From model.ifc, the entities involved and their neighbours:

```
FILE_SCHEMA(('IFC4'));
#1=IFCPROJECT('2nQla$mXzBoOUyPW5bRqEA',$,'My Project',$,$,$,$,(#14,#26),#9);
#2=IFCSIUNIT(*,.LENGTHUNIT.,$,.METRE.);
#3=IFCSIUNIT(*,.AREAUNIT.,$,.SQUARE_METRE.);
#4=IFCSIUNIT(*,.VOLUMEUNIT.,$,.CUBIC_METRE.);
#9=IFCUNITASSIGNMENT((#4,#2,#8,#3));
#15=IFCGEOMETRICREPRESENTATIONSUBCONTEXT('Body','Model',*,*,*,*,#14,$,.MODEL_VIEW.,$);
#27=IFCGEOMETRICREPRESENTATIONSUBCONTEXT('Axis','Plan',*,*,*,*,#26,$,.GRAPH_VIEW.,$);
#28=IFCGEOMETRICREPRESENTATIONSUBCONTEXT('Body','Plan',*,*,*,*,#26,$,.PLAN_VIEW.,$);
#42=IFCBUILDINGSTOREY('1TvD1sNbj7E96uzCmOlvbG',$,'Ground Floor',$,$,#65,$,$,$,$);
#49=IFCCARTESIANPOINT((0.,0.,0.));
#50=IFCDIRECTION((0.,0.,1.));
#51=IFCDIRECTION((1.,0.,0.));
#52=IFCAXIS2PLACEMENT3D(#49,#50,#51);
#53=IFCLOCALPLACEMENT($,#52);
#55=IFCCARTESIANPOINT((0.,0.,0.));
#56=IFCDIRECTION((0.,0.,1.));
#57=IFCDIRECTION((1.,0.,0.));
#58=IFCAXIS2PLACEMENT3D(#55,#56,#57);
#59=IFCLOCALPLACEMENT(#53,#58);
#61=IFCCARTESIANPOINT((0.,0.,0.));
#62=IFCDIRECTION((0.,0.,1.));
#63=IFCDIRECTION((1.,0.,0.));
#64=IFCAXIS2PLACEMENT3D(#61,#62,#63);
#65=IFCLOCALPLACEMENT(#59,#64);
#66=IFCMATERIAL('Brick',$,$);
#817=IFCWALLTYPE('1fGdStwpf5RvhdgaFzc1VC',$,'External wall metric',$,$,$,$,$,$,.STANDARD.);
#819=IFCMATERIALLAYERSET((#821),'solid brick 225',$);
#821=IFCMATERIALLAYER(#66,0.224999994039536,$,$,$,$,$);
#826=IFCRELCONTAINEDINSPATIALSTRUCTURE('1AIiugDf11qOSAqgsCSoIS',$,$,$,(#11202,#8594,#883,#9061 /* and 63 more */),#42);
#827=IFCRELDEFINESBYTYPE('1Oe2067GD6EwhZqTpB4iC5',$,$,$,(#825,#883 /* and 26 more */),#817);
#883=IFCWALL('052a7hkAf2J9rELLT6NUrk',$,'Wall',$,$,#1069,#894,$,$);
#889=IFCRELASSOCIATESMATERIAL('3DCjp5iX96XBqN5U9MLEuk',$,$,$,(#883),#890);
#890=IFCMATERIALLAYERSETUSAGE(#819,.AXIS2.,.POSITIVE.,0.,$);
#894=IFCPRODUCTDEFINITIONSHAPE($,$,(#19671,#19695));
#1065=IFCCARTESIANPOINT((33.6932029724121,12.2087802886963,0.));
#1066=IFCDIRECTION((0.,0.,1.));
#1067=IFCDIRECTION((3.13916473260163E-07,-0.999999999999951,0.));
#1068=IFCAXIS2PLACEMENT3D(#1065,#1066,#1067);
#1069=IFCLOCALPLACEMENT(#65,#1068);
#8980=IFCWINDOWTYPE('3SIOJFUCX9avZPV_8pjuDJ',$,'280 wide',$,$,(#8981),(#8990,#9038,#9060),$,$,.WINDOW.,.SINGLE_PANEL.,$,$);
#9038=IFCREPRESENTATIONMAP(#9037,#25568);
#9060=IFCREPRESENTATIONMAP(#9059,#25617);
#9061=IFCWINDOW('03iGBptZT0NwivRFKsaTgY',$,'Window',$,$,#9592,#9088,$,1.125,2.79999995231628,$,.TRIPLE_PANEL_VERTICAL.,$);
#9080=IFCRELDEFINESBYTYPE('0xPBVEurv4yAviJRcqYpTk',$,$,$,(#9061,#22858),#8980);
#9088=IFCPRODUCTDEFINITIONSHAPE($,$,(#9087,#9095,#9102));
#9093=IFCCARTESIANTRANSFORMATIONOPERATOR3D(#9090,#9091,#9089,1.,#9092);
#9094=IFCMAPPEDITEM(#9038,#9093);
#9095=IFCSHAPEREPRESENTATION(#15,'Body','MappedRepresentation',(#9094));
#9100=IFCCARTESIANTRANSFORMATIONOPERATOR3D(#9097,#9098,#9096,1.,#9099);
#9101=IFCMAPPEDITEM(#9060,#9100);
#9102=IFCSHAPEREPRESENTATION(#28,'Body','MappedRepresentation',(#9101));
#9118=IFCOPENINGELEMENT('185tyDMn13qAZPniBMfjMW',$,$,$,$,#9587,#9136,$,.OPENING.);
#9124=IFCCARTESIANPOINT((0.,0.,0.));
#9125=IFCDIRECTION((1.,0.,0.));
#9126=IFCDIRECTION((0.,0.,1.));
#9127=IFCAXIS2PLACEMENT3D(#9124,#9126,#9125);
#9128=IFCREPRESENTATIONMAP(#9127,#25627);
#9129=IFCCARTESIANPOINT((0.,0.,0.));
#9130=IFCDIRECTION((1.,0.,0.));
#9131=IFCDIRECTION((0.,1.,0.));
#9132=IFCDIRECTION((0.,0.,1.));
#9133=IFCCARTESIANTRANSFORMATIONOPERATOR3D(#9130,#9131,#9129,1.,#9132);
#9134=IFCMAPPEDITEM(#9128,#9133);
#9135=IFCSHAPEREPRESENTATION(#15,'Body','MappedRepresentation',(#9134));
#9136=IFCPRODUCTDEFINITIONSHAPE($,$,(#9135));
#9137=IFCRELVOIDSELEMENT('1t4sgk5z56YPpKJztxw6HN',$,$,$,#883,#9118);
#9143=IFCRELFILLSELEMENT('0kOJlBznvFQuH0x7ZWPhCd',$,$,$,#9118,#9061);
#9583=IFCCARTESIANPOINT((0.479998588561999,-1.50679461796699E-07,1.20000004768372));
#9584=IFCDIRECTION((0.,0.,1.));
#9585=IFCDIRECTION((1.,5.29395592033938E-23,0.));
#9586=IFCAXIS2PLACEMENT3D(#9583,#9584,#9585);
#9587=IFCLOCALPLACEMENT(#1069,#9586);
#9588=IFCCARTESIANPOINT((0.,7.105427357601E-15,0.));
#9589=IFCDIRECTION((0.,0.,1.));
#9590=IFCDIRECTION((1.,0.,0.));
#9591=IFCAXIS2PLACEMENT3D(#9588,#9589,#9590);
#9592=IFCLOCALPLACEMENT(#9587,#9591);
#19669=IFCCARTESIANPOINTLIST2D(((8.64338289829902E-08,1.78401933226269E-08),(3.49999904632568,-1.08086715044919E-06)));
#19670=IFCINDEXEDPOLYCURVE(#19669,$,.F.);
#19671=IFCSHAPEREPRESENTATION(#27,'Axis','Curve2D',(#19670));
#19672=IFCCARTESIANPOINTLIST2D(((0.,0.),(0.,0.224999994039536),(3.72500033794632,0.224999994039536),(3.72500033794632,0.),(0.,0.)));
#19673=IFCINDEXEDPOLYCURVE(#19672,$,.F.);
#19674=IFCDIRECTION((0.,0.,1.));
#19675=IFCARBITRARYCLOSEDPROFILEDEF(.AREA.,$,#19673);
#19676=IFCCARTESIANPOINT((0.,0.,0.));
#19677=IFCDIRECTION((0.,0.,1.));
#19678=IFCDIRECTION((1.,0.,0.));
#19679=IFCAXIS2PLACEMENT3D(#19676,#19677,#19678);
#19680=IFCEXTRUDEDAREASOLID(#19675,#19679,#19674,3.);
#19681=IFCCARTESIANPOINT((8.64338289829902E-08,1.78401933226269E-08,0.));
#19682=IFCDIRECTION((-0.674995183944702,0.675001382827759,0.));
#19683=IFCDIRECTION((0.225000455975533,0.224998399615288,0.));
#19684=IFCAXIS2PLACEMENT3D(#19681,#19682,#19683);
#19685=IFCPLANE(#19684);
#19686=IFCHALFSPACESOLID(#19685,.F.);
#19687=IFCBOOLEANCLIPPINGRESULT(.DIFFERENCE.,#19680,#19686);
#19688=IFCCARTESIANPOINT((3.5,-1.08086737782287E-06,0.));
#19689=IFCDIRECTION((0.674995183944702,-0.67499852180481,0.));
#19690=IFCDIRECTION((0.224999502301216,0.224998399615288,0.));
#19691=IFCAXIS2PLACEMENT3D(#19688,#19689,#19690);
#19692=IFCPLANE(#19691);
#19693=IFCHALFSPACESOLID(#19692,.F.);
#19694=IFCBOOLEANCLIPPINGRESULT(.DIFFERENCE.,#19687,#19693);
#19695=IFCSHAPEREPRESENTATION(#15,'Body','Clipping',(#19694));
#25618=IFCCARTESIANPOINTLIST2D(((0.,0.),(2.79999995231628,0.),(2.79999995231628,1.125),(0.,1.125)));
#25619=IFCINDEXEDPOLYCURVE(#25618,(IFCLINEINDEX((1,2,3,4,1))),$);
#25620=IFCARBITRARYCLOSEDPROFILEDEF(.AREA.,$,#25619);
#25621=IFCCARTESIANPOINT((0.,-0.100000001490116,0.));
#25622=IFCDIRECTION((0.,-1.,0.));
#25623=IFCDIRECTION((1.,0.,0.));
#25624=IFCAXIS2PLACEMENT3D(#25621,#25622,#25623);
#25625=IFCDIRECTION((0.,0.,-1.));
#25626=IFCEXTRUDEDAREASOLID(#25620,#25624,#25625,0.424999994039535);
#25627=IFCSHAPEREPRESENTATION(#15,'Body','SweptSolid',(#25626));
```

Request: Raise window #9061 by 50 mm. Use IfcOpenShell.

```python
import numpy as np
import ifcopenshell
import ifcopenshell.api.geometry
import ifcopenshell.util.placement
import ifcopenshell.util.unit

model = ifcopenshell.open("model.ifc")
unit_scale = ifcopenshell.util.unit.calculate_unit_scale(model)

window = model.by_id(9061)
opening = window.FillsVoids[0].RelatingOpeningElement
dz = 0.05 / unit_scale

shift = np.array([0.0, 0.0, dz])
# The window is placed relative to its opening, so it follows when the opening moves.
matrix = ifcopenshell.util.placement.get_local_placement(opening.ObjectPlacement)
matrix[:3, 3] += shift
ifcopenshell.api.geometry.edit_object_placement(
    model, product=opening, matrix=matrix, is_si=False, should_transform_children=True
)

print(f"moved by {dz * unit_scale:+.3f} m")

model.write("model-out.ifc")
```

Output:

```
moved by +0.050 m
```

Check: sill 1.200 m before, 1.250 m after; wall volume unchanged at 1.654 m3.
